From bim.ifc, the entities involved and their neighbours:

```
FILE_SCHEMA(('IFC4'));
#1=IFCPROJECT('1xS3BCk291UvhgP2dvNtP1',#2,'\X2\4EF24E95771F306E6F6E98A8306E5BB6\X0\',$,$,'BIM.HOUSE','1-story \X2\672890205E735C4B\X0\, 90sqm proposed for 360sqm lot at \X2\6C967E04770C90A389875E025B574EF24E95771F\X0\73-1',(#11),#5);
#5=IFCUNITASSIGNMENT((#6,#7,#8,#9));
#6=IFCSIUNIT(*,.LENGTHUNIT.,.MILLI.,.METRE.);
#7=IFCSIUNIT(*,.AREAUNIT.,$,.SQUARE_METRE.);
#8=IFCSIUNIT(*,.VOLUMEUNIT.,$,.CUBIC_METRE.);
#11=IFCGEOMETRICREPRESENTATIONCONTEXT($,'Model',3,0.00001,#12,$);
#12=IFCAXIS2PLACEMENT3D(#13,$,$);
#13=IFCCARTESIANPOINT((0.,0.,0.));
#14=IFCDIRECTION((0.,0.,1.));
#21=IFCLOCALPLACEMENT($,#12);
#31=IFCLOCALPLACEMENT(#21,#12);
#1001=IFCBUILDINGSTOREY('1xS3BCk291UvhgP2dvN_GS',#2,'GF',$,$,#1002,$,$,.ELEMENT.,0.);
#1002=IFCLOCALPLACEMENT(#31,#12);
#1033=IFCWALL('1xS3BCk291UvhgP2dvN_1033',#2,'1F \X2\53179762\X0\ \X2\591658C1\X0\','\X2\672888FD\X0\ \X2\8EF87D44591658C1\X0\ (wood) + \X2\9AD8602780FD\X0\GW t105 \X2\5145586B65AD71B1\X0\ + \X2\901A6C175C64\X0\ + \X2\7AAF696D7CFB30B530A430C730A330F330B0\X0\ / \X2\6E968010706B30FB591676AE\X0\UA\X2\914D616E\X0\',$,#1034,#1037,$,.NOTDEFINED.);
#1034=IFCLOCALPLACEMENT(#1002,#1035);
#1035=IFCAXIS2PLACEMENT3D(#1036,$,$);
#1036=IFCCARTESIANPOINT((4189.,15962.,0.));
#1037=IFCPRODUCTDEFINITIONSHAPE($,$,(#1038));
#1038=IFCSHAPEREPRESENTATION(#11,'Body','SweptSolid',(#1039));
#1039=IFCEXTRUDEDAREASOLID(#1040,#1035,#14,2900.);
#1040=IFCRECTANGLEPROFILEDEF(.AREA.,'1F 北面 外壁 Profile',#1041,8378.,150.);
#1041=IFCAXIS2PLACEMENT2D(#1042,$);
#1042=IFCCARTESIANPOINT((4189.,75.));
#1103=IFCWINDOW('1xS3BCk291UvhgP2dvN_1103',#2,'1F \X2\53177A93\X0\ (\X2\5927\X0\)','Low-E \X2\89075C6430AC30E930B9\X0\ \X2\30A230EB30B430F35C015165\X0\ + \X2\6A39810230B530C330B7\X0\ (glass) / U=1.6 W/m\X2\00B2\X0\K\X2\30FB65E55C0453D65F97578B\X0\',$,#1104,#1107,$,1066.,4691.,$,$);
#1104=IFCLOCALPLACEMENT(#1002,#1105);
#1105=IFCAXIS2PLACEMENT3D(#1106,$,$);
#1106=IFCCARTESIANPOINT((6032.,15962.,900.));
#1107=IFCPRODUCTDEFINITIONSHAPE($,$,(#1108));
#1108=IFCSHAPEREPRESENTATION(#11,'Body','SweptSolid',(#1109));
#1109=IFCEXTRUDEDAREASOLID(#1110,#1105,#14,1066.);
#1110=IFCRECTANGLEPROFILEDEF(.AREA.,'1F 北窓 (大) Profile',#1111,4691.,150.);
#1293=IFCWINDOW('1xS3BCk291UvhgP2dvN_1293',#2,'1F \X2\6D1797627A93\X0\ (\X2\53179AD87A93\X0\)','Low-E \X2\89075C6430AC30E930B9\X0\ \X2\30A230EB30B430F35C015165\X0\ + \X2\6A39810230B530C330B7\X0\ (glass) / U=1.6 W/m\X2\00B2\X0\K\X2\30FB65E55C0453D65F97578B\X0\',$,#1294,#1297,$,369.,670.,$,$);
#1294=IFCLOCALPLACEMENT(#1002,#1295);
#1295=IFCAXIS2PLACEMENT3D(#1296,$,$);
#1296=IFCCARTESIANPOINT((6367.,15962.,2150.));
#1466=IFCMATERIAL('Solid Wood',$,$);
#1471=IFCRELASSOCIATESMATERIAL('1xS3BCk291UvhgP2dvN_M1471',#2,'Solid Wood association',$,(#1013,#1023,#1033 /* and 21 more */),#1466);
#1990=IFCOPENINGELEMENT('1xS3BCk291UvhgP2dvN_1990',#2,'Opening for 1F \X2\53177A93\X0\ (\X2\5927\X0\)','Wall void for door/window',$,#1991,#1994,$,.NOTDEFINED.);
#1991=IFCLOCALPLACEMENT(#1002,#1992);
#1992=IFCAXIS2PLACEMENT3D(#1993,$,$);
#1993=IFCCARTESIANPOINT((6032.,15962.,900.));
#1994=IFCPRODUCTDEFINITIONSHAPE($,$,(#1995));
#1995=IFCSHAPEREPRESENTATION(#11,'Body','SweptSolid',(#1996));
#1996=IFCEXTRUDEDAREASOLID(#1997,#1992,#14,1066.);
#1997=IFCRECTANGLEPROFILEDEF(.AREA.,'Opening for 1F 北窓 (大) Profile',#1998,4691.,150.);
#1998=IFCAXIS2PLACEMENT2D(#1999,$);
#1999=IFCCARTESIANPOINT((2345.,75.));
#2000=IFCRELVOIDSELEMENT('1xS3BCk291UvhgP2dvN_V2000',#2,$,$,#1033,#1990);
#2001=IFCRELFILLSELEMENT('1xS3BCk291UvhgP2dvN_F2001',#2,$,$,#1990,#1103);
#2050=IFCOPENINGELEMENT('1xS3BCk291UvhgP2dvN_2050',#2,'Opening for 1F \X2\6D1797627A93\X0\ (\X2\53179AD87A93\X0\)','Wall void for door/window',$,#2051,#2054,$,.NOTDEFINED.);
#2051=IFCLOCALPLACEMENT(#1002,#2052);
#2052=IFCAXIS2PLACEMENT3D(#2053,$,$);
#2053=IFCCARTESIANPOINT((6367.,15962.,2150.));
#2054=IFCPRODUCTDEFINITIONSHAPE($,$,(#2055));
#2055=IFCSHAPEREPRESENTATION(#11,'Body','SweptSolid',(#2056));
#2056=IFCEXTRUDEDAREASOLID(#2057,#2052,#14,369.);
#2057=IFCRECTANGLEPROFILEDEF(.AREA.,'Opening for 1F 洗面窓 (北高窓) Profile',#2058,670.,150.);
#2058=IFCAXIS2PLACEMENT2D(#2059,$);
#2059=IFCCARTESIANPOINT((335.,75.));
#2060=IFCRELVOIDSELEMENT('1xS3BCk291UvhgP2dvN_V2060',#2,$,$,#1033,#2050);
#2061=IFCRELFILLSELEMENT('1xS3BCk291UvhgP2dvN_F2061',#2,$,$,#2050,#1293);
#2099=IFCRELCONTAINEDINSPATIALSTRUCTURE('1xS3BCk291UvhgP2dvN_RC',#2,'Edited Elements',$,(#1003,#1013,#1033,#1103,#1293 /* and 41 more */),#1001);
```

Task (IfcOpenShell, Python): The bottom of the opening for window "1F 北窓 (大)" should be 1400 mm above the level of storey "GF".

```python
import numpy as np
import ifcopenshell
import ifcopenshell.api.geometry
import ifcopenshell.geom
import ifcopenshell.util.element
import ifcopenshell.util.placement
import ifcopenshell.util.shape
import ifcopenshell.util.unit

model = ifcopenshell.open("bim.ifc")
unit_scale = ifcopenshell.util.unit.calculate_unit_scale(model)

window = model.by_id(1103)
opening = window.FillsVoids[0].RelatingOpeningElement
storey = ifcopenshell.util.element.get_container(window, ifc_class="IfcBuildingStorey")
level = ifcopenshell.util.placement.get_local_placement(storey.ObjectPlacement)[2, 3]

# The opening's origin need not be at the sill, so measure its lowest point.
shape = ifcopenshell.geom.create_shape(ifcopenshell.geom.settings(), opening)
bottom = ifcopenshell.util.shape.get_shape_bottom_elevation(shape, shape.geometry) / unit_scale
dz = level + 1.4 / unit_scale - bottom

shift = np.array([0.0, 0.0, dz])
# The window is not placed relative to its opening, so move both.
for product in (opening, window):
    matrix = ifcopenshell.util.placement.get_local_placement(product.ObjectPlacement)
    matrix[:3, 3] += shift
    ifcopenshell.api.geometry.edit_object_placement(model, product=product, matrix=matrix, is_si=False)

print(f"moved by {dz * unit_scale:+.3f} m")

model.write("bim_edited.ifc")
```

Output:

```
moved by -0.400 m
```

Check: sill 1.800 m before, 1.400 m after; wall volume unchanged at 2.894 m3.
